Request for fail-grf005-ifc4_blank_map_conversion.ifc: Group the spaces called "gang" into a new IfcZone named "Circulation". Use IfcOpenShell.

First a look at what the model holds.

```python
import ifcopenshell

model = ifcopenshell.open("fail-grf005-ifc4_blank_map_conversion.ifc")
print(model.schema)
seen = {}
for space in model.by_type("IfcSpace"):
    seen[space.LongName] = seen.get(space.LongName, 0) + 1
for name, count in sorted(seen.items(), key=str):
    print(count, "x", name)
print("zones:", [z.Name for z in model.by_type("IfcZone")][:20])
```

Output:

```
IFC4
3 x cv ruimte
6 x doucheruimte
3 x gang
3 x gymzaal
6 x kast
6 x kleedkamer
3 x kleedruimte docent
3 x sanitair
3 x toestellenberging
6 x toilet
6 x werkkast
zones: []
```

```python
import ifcopenshell
import ifcopenshell.api.group
import ifcopenshell.api.root

model = ifcopenshell.open("fail-grf005-ifc4_blank_map_conversion.ifc")

names = {"gang"}
spaces = [s for s in model.by_type("IfcSpace") if s.LongName in names]

zone = ifcopenshell.api.root.create_entity(model, ifc_class="IfcZone", name="Circulation")
ifcopenshell.api.group.assign_group(model, products=spaces, group=zone)
print(len(spaces), "spaces in", zone.Name)

model.write("fail-grf005-ifc4_blank_map_conversion-out.ifc")
```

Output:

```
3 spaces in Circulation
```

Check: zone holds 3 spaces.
